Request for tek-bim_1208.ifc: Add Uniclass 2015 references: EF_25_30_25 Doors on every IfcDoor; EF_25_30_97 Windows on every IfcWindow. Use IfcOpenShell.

First a look at what the model holds.

```python
import ifcopenshell

model = ifcopenshell.open("tek-bim_1208.ifc")
print(model.schema)
print("classifications:", [c.Name for c in model.by_type("IfcClassification")])
for ifc_class in ("IfcDoor", "IfcRoof", "IfcStair", "IfcWall", "IfcWindow"):
    print(ifc_class, len(model.by_type(ifc_class)))
```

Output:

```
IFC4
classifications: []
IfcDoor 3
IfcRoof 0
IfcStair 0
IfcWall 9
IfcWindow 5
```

```python
import ifcopenshell
import ifcopenshell.api.classification

model = ifcopenshell.open("tek-bim_1208.ifc")

system = ifcopenshell.api.classification.add_classification(model, classification="Uniclass 2015")

codes = {
    "IfcDoor": ("EF_25_30_25", "Doors"),
    "IfcWindow": ("EF_25_30_97", "Windows"),
}
for ifc_class, (code, name) in codes.items():
    products = model.by_type(ifc_class)
    ifcopenshell.api.classification.add_reference(
        model, products=products, classification=system, identification=code, name=name
    )
    print(code, len(products))

model.write("tek-bim_1208_v2.ifc")
```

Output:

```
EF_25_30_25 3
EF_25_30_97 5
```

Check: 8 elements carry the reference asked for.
